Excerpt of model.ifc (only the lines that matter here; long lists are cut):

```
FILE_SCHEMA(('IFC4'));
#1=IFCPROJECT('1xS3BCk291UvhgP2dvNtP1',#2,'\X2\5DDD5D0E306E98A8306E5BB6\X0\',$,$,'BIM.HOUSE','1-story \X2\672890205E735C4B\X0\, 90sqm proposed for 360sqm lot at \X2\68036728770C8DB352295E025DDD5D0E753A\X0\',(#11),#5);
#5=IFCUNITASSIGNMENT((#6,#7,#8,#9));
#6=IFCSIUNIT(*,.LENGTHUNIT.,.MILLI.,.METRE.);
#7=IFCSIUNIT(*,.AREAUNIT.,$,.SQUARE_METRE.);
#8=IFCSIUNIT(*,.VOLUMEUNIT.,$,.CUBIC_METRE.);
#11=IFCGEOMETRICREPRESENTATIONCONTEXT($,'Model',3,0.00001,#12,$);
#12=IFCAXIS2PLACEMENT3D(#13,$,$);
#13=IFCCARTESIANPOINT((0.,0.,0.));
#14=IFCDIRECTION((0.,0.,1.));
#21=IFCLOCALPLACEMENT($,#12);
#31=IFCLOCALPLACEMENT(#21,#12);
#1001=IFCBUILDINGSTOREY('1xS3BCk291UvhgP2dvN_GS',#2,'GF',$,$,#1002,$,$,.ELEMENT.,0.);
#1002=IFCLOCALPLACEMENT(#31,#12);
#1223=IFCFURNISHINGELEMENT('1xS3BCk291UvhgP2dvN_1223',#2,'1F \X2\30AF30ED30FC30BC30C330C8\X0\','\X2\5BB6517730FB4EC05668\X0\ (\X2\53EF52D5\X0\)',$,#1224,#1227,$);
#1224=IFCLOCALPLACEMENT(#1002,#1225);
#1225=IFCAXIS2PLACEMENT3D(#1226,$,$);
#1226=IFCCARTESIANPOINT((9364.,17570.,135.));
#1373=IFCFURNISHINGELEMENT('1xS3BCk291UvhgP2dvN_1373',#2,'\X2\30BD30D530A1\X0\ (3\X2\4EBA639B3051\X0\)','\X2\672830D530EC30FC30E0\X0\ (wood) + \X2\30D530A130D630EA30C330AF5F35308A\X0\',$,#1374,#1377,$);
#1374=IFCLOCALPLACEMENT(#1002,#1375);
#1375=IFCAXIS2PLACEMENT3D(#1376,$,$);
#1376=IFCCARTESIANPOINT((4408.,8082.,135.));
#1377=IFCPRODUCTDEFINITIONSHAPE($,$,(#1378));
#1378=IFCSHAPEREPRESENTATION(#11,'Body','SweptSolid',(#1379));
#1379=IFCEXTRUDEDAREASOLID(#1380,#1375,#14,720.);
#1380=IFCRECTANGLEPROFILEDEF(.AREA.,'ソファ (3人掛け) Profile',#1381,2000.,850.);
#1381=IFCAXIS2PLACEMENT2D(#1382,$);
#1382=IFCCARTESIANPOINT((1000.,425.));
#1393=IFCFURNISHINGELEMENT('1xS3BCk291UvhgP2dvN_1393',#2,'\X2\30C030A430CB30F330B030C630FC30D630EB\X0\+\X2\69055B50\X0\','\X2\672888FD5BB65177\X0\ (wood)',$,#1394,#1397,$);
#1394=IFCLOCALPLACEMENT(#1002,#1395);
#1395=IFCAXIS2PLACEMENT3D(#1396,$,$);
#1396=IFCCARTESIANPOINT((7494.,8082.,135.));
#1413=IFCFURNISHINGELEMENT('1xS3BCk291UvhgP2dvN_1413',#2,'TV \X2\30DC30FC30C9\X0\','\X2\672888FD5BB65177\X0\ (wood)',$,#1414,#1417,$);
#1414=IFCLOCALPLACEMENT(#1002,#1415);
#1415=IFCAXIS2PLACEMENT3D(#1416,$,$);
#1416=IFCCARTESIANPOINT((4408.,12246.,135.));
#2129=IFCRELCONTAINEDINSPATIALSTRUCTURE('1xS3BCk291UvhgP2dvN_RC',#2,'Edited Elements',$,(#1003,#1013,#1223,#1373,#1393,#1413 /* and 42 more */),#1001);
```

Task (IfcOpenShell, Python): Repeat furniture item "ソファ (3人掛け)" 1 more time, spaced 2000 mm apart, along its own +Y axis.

```python
import ifcopenshell
import ifcopenshell.api.geometry
import ifcopenshell.api.root
import ifcopenshell.util.element
import ifcopenshell.util.placement

model = ifcopenshell.open("model.ifc")


def reuse_history(source, copy):
    """copy_class also copies each property set's owner history, people and application; keep the originals."""
    for rel in copy.IsDefinedBy:
        if rel.is_a("IfcRelDefinesByProperties") and (history := rel.RelatingPropertyDefinition.OwnerHistory):
            rel.RelatingPropertyDefinition.OwnerHistory = source.OwnerHistory
            ifcopenshell.util.element.remove_deep2(model, history)


source = model.by_id(1373)
base = ifcopenshell.util.placement.get_local_placement(source.ObjectPlacement)
step = base[:3, 1] * 2000.0

for i in range(1, 2):
    copy = ifcopenshell.api.root.copy_class(model, product=source)
    copy.Representation = ifcopenshell.util.element.copy_deep(
        model, source.Representation, exclude=["IfcGeometricRepresentationContext", "IfcRepresentationMap"]
    )
    reuse_history(source, copy)
    matrix = base.copy()
    matrix[:3, 3] += i * step
    print("added at", matrix[:3, 3].round(3) + 0.0)
    ifcopenshell.api.geometry.edit_object_placement(model, product=copy, matrix=matrix, is_si=False)

model.write("model_v2.ifc")
```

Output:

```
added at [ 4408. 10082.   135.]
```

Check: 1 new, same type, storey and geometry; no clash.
